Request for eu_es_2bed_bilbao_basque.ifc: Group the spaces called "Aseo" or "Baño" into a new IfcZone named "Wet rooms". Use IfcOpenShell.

First a look at what the model holds.

```python
import ifcopenshell

model = ifcopenshell.open("eu_es_2bed_bilbao_basque.ifc")
print(model.schema)
seen = {}
for space in model.by_type("IfcSpace"):
    seen[space.LongName] = seen.get(space.LongName, 0) + 1
for name, count in sorted(seen.items(), key=str):
    print(count, "x", name)
print("zones:", [z.Name for z in model.by_type("IfcZone")][:20])
```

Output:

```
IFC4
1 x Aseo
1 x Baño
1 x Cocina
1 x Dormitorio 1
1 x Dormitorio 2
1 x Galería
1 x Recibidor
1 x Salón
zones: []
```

```python
import ifcopenshell
import ifcopenshell.api.group
import ifcopenshell.api.root

model = ifcopenshell.open("eu_es_2bed_bilbao_basque.ifc")

names = {"Aseo", "Baño"}
spaces = [s for s in model.by_type("IfcSpace") if s.LongName in names]

zone = ifcopenshell.api.root.create_entity(model, ifc_class="IfcZone", name="Wet rooms")
ifcopenshell.api.group.assign_group(model, products=spaces, group=zone)
print(len(spaces), "spaces in", zone.Name)

model.write("eu_es_2bed_bilbao_basque-out.ifc")
```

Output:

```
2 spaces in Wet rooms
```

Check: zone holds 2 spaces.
